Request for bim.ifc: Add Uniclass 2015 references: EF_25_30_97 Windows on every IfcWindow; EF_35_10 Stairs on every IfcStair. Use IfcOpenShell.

First a look at what the model holds.

```python
import ifcopenshell

model = ifcopenshell.open("bim.ifc")
print(model.schema)
print("classifications:", [c.Name for c in model.by_type("IfcClassification")])
for ifc_class in ("IfcDoor", "IfcRoof", "IfcStair", "IfcWall", "IfcWindow"):
    print(ifc_class, len(model.by_type(ifc_class)))
```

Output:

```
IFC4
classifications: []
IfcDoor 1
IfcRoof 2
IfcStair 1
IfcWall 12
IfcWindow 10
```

```python
import ifcopenshell
import ifcopenshell.api.classification

model = ifcopenshell.open("bim.ifc")

system = ifcopenshell.api.classification.add_classification(model, classification="Uniclass 2015")

codes = {
    "IfcWindow": ("EF_25_30_97", "Windows"),
    "IfcStair": ("EF_35_10", "Stairs"),
}
for ifc_class, (code, name) in codes.items():
    products = model.by_type(ifc_class)
    ifcopenshell.api.classification.add_reference(
        model, products=products, classification=system, identification=code, name=name
    )
    print(code, len(products))

model.write("bim-out.ifc")
```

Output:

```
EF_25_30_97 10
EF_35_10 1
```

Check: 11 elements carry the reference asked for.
